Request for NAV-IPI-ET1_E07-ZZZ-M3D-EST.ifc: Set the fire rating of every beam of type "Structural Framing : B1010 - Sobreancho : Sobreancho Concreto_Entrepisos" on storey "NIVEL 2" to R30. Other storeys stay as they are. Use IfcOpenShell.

First a look at what the model holds.

```python
import ifcopenshell
import ifcopenshell.util.element

model = ifcopenshell.open("NAV-IPI-ET1_E07-ZZZ-M3D-EST.ifc")
print(model.schema)
storey = next(s for s in model.by_type("IfcBuildingStorey") if s.Name == "NIVEL 2")
beams = [e for e in ifcopenshell.util.element.get_decomposition(storey) if e.is_a("IfcBeam")]
seen = {}
for e in beams:
    element_type = ifcopenshell.util.element.get_type(e)
    key = (element_type.Name if element_type != e and element_type else None, ifcopenshell.util.element.get_pset(e, "Pset_BeamCommon", "FireRating"))
    seen[key] = seen.get(key, 0) + 1
for (name, value), count in sorted(seen.items(), key=str):
    print(count, "x", name, "|", value)
```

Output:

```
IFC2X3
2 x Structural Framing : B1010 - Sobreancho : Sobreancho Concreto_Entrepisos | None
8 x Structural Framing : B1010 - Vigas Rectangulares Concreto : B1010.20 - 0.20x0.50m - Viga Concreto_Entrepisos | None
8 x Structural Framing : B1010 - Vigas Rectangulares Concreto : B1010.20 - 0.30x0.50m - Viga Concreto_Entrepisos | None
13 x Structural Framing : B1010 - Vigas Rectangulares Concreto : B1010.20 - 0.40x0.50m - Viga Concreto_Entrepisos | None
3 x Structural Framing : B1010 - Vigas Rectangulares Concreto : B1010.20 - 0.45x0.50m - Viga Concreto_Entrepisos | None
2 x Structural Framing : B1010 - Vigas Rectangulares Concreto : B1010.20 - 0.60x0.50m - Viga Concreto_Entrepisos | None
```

```python
import ifcopenshell
import ifcopenshell.api.pset
import ifcopenshell.util.element

model = ifcopenshell.open("NAV-IPI-ET1_E07-ZZZ-M3D-EST.ifc")

storey = next(s for s in model.by_type("IfcBuildingStorey") if s.Name == "NIVEL 2")
beams = [e for e in ifcopenshell.util.element.get_decomposition(storey) if e.is_a("IfcBeam")]

count = 0
for e in beams:
    element_type = ifcopenshell.util.element.get_type(e)
    if element_type in (None, e) or element_type.Name != "Structural Framing : B1010 - Sobreancho : Sobreancho Concreto_Entrepisos":
        continue
    # add_pset returns the element's existing set when there is one.
    pset = ifcopenshell.api.pset.add_pset(model, product=e, name="Pset_BeamCommon")
    ifcopenshell.api.pset.edit_pset(model, pset=pset, properties={"FireRating": "R30"})
    count += 1

print(count, "beams updated")

model.write("NAV-IPI-ET1_E07-ZZZ-M3D-EST_v2.ifc")
```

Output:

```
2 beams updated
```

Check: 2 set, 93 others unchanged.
